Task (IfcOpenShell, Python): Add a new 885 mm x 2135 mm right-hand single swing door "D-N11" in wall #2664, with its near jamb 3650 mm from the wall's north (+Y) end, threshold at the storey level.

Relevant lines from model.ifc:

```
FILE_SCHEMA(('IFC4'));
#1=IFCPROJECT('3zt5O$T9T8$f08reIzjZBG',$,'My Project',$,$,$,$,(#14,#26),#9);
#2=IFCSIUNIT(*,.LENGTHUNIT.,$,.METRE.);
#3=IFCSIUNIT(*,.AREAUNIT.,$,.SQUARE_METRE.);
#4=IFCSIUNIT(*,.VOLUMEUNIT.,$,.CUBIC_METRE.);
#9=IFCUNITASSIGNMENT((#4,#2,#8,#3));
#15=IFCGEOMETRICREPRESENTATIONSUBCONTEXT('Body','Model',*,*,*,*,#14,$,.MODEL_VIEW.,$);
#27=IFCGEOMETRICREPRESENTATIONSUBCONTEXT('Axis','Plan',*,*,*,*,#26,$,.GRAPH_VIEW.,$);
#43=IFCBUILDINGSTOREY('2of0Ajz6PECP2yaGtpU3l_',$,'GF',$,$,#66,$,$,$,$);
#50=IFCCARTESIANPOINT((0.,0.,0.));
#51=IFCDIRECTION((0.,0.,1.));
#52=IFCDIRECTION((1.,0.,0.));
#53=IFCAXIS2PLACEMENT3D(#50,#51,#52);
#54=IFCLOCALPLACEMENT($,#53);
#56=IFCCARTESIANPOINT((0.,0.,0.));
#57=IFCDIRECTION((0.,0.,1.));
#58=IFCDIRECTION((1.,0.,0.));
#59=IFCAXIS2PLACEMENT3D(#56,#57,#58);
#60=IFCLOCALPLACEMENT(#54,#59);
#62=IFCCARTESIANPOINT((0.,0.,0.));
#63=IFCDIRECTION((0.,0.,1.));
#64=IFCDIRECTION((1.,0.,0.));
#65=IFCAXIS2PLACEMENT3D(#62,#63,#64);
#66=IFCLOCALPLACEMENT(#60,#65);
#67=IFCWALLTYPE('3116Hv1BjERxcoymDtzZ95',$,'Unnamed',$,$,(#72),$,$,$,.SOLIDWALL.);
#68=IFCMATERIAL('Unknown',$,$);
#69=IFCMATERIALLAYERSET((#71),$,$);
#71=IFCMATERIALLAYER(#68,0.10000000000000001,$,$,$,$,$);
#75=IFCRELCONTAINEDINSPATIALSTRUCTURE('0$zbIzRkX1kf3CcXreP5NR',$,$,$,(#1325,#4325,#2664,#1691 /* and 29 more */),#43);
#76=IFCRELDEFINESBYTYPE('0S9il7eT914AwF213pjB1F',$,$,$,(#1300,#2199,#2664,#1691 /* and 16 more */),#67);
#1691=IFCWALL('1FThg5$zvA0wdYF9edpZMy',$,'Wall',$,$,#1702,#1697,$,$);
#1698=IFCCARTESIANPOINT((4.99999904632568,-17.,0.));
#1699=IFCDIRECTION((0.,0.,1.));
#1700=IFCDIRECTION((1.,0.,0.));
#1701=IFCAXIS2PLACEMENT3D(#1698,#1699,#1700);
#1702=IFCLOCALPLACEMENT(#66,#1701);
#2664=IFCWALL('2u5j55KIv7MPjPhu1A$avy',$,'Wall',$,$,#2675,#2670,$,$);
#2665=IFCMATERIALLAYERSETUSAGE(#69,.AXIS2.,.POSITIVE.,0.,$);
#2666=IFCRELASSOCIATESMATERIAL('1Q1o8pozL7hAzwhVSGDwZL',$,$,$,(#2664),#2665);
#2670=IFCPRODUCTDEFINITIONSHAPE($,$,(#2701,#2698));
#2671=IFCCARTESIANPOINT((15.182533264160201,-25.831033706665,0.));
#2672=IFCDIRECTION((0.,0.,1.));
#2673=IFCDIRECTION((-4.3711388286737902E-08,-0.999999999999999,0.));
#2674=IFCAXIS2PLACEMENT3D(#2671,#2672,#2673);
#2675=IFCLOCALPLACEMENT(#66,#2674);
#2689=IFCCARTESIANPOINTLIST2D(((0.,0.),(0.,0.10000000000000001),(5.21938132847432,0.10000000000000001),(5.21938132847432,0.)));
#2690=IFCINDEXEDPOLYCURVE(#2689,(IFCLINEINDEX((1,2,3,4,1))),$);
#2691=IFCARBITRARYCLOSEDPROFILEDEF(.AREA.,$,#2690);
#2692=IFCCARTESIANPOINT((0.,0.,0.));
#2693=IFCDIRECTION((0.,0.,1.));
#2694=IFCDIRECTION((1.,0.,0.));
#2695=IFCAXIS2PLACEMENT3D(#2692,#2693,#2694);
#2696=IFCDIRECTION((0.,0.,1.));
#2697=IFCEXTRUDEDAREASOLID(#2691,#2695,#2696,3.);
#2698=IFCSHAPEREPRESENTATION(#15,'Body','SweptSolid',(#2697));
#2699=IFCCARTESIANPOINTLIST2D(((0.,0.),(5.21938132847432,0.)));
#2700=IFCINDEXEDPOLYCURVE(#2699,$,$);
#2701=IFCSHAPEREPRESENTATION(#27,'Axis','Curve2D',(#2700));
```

```python
import numpy as np
import ifcopenshell
import ifcopenshell.api.feature
import ifcopenshell.api.geometry
import ifcopenshell.api.root
import ifcopenshell.api.spatial
import ifcopenshell.geom
import ifcopenshell.util.element
import ifcopenshell.util.placement
import ifcopenshell.util.representation
import ifcopenshell.util.shape
import ifcopenshell.util.unit

model = ifcopenshell.open("model.ifc")
unit_scale = ifcopenshell.util.unit.calculate_unit_scale(model)
settings = ifcopenshell.geom.settings()


def volume(element):
    """Net volume in cubic metres, openings subtracted."""
    shape = ifcopenshell.geom.create_shape(settings, element)
    return ifcopenshell.util.shape.get_volume(shape.geometry)


wall = model.by_id(2664)
storey = ifcopenshell.util.element.get_container(wall, ifc_class="IfcBuildingStorey")
context = ifcopenshell.util.representation.get_context(model, "Model", "Body", "MODEL_VIEW")
before = volume(wall)

width, height, from_end, sill = 0.885, 2.135, 3.65, 0.0  # metres

# The wall runs along its own X axis, and the end named is its -X end.
wall_shape = ifcopenshell.geom.create_shape(settings, wall)
x, y, z = ifcopenshell.util.shape.get_vertices(wall_shape.geometry).T
start = x.min() + from_end
face, thickness = float(y.min()), float(y.max() - y.min())
wall_matrix = ifcopenshell.util.placement.get_local_placement(wall.ObjectPlacement)
level = ifcopenshell.util.placement.get_local_placement(storey.ObjectPlacement)[2, 3]


def in_wall(x, y):
    """Placement at x, y metres in the wall's axes, at sill height."""
    matrix = wall_matrix.copy()
    matrix[:, 3] = wall_matrix @ np.array([x / unit_scale, y / unit_scale, 0.0, 1.0])
    matrix[2, 3] = level + sill / unit_scale
    return matrix


# Opening: a box that overshoots both wall faces by 50 mm.
opening = ifcopenshell.api.root.create_entity(model, ifc_class="IfcOpeningElement", predefined_type="OPENING")
box = ifcopenshell.api.geometry.add_wall_representation(
    model, context=context, length=width, height=height, thickness=thickness + 0.1
)
ifcopenshell.api.geometry.assign_representation(model, product=opening, representation=box)
ifcopenshell.api.geometry.edit_object_placement(model, product=opening, matrix=in_wall(start, face - 0.05), is_si=False)
ifcopenshell.api.feature.add_feature(model, feature=opening, element=wall)

door = ifcopenshell.api.root.create_entity(model, ifc_class="IfcDoor", name="D-N11", predefined_type="DOOR")
door.OverallWidth, door.OverallHeight = width / unit_scale, height / unit_scale
door.OperationType = "SINGLE_SWING_RIGHT"
body = ifcopenshell.api.geometry.add_door_representation(
    model,
    context=context,
    overall_width=door.OverallWidth,
    overall_height=door.OverallHeight,
    operation_type="SINGLE_SWING_RIGHT",
    lining_properties={"LiningDepth": thickness / unit_scale, "ThresholdDepth": thickness / unit_scale},
)
ifcopenshell.api.geometry.assign_representation(model, product=door, representation=body)
ifcopenshell.api.spatial.assign_container(model, products=[door], relating_structure=storey)
ifcopenshell.api.feature.add_filling(model, opening=opening, element=door)

# The lining spans the wall, so the door starts at the wall face.
ifcopenshell.api.geometry.edit_object_placement(model, product=door, matrix=in_wall(start, face), is_si=False)

after = volume(wall)

print(f"wall volume {before:.3f} -> {after:.3f} m3")

model.write("model_v2.ifc")
```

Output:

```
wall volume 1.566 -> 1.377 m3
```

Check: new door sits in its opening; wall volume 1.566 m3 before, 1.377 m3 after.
